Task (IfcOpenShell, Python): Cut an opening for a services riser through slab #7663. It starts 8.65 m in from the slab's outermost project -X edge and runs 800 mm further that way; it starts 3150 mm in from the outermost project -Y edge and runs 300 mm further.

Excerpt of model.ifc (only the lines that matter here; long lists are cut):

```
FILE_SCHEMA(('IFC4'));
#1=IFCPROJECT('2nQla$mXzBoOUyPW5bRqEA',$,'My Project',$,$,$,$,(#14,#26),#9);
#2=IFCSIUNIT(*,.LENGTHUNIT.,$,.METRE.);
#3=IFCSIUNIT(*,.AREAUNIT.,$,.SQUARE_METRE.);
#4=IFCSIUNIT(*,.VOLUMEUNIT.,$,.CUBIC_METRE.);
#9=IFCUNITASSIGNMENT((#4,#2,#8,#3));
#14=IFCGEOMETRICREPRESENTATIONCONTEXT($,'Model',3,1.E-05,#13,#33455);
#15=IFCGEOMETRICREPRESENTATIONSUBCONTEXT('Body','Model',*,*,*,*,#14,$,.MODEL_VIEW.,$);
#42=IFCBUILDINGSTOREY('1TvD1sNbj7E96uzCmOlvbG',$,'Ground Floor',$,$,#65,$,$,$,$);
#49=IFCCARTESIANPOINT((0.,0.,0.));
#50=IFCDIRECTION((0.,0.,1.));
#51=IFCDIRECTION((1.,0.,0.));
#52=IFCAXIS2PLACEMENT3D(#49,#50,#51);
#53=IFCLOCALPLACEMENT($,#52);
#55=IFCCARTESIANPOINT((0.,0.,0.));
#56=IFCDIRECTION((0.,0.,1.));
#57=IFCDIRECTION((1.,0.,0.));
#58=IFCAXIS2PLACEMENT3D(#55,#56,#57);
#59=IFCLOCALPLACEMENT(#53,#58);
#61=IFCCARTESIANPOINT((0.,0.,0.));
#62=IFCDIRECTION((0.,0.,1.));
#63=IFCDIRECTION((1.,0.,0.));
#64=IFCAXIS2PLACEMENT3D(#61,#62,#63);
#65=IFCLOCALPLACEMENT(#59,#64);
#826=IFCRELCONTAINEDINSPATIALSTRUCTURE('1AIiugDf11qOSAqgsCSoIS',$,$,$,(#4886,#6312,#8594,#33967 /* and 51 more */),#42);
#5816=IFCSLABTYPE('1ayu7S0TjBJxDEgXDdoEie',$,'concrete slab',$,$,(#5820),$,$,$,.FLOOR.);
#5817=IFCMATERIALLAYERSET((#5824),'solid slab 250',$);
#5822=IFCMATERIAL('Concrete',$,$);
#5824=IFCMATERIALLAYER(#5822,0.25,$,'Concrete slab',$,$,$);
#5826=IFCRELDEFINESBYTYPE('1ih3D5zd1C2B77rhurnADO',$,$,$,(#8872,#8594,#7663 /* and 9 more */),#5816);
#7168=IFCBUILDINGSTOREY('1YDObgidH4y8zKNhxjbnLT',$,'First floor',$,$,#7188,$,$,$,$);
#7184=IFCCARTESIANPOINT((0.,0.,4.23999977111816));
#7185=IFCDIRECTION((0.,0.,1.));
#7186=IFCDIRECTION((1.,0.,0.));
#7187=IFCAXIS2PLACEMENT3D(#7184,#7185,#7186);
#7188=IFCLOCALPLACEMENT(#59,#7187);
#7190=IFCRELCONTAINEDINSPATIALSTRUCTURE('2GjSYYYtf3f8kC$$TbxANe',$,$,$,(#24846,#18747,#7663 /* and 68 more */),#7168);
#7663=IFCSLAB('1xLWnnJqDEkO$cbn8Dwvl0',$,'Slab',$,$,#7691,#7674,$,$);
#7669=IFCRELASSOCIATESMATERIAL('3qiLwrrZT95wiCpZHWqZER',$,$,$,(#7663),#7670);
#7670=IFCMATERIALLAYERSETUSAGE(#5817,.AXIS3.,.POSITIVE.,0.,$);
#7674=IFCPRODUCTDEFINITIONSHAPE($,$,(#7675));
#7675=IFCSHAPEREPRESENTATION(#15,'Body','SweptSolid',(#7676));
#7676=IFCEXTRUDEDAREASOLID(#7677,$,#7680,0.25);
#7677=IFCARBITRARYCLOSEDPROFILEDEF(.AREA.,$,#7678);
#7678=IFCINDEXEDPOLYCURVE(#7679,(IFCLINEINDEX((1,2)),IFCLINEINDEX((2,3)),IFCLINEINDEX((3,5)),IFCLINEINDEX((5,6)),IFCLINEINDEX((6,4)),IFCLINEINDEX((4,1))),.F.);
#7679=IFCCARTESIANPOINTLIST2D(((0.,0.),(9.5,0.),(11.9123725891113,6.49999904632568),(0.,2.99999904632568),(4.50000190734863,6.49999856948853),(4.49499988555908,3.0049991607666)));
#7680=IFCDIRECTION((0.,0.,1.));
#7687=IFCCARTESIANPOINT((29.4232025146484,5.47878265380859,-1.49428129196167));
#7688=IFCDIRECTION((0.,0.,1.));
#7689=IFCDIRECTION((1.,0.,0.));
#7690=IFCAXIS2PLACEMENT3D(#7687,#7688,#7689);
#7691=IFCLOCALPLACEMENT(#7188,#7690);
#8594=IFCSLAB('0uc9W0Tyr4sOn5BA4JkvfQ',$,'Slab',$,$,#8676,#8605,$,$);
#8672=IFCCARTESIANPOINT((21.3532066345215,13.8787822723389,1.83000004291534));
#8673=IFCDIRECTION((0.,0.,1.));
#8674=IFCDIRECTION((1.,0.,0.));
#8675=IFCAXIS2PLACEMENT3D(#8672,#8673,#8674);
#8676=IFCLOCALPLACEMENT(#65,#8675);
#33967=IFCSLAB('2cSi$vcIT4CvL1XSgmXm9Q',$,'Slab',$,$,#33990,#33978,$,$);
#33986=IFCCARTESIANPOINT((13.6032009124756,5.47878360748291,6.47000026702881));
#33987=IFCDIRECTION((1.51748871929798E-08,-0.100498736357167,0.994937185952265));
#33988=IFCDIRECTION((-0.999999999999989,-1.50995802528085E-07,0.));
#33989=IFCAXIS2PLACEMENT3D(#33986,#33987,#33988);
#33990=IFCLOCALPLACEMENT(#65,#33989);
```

```python
import numpy as np
import ifcopenshell
import ifcopenshell.api.feature
import ifcopenshell.api.geometry
import ifcopenshell.api.root
import ifcopenshell.geom
import ifcopenshell.util.placement
import ifcopenshell.util.representation
import ifcopenshell.util.shape
import ifcopenshell.util.unit

model = ifcopenshell.open("model.ifc")
unit_scale = ifcopenshell.util.unit.calculate_unit_scale(model)
settings = ifcopenshell.geom.settings()


def volume(element):
    """Net volume in cubic metres, openings subtracted."""
    shape = ifcopenshell.geom.create_shape(settings, element)
    return ifcopenshell.util.shape.get_volume(shape.geometry)


slab = model.by_guid("1xLWnnJqDEkO$cbn8Dwvl0")
before = volume(slab)

# Extent in the slab's own axes, in metres. The edges named are its -X and -Y sides.
slab_shape = ifcopenshell.geom.create_shape(settings, slab)
vertices = ifcopenshell.util.shape.get_vertices(slab_shape.geometry)
x_min, y_min, bottom = vertices.min(axis=0)
top = vertices[:, 2].max()

opening = ifcopenshell.api.root.create_entity(model, ifc_class="IfcOpeningElement", name="Services riser opening", predefined_type="OPENING")
context = ifcopenshell.util.representation.get_context(model, "Model", "Body", "MODEL_VIEW")
width, depth = 0.8, 0.3
outline = [(0.0, 0.0), (width, 0.0), (width, depth), (0.0, depth), (0.0, 0.0)]
# Overshoot both faces by 50 mm so the cut is clean.
shape = ifcopenshell.api.geometry.add_slab_representation(
    model, context=context, depth=top - bottom + 0.1, polyline=outline
)
ifcopenshell.api.geometry.assign_representation(model, product=opening, representation=shape)

matrix = ifcopenshell.util.placement.get_local_placement(slab.ObjectPlacement)
matrix[:, 3] = matrix @ np.append(np.array([x_min + 8.65, y_min + 3.15, bottom - 0.05]) / unit_scale, 1.0)
ifcopenshell.api.geometry.edit_object_placement(model, product=opening, matrix=matrix, is_si=False)
ifcopenshell.api.feature.add_feature(model, feature=opening, element=slab)

after = volume(slab)

print(f"slab volume {before:.3f} -> {after:.3f} m3")

model.write("model_rev.ifc")
```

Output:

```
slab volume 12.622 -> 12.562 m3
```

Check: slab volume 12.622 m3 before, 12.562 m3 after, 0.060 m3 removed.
